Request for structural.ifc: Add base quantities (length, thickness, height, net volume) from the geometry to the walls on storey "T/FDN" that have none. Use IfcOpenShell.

First a look at what the model holds.

```python
import ifcopenshell
import ifcopenshell.util.element
import ifcopenshell.util.unit

model = ifcopenshell.open("structural.ifc")
print(model.schema)
for unit_type in ("LENGTHUNIT", "AREAUNIT", "VOLUMEUNIT"):
    print(unit_type, ifcopenshell.util.unit.calculate_unit_scale(model, unit_type))
storey = next(s for s in model.by_type("IfcBuildingStorey") if s.Name == "T/FDN")
walls = [e for e in ifcopenshell.util.element.get_decomposition(storey) if e.is_a("IfcWall")]
for e in sorted(walls, key=lambda e: e.id()):
    print(e.id(), e.is_a(), e.Name, list(ifcopenshell.util.element.get_psets(e, qtos_only=True)), sep=" | ")
```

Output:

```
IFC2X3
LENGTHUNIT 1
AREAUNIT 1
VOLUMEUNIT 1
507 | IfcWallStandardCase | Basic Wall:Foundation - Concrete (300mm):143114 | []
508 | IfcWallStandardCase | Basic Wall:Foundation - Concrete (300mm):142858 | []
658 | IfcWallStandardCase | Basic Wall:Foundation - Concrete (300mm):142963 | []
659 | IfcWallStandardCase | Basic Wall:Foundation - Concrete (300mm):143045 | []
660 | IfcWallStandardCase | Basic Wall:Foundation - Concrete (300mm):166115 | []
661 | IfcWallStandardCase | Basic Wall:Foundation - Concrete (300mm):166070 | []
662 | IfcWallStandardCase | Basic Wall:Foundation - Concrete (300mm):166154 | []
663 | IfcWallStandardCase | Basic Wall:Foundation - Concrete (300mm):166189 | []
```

```python
import ifcopenshell
import ifcopenshell.api.pset
import ifcopenshell.geom
import ifcopenshell.util.element
import ifcopenshell.util.shape
import ifcopenshell.util.unit

model = ifcopenshell.open("structural.ifc")
unit_scale = ifcopenshell.util.unit.calculate_unit_scale(model)
volume_scale = ifcopenshell.util.unit.calculate_unit_scale(model, "VOLUMEUNIT")
settings = ifcopenshell.geom.settings()

storey = next(s for s in model.by_type("IfcBuildingStorey") if s.Name == "T/FDN")
walls = [e for e in ifcopenshell.util.element.get_decomposition(storey) if e.is_a("IfcWall")]

for e in sorted(walls, key=lambda e: e.id()):
    if ifcopenshell.util.element.get_psets(e, qtos_only=True, should_inherit=False):
        continue
    # Geometry comes back in metres, in the element's own axes.
    shape = ifcopenshell.geom.create_shape(settings, e)
    values = {
        "Length": ifcopenshell.util.shape.get_x(shape.geometry) / unit_scale,
        "Width": ifcopenshell.util.shape.get_y(shape.geometry) / unit_scale,
        "Height": ifcopenshell.util.shape.get_z(shape.geometry) / unit_scale,
        "NetVolume": ifcopenshell.util.shape.get_volume(shape.geometry) / volume_scale,
    }
    qto = ifcopenshell.api.pset.add_qto(model, product=e, name="BaseQuantities")
    ifcopenshell.api.pset.edit_qto(model, qto=qto, properties=values)
    print(e.id(), {k: round(v, 3) for k, v in values.items()})

model.write("structural_updated.ifc")
```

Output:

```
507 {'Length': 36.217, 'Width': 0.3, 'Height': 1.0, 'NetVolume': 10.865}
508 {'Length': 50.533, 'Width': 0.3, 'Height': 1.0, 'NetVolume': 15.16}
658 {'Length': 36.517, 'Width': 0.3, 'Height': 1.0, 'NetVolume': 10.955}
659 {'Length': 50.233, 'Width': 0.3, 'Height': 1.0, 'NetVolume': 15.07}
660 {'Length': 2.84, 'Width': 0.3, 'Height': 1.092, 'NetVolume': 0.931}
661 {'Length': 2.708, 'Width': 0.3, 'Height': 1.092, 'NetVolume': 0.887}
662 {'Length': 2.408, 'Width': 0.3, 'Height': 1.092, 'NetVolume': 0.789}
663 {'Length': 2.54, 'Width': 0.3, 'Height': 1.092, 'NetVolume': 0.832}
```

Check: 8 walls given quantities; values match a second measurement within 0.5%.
